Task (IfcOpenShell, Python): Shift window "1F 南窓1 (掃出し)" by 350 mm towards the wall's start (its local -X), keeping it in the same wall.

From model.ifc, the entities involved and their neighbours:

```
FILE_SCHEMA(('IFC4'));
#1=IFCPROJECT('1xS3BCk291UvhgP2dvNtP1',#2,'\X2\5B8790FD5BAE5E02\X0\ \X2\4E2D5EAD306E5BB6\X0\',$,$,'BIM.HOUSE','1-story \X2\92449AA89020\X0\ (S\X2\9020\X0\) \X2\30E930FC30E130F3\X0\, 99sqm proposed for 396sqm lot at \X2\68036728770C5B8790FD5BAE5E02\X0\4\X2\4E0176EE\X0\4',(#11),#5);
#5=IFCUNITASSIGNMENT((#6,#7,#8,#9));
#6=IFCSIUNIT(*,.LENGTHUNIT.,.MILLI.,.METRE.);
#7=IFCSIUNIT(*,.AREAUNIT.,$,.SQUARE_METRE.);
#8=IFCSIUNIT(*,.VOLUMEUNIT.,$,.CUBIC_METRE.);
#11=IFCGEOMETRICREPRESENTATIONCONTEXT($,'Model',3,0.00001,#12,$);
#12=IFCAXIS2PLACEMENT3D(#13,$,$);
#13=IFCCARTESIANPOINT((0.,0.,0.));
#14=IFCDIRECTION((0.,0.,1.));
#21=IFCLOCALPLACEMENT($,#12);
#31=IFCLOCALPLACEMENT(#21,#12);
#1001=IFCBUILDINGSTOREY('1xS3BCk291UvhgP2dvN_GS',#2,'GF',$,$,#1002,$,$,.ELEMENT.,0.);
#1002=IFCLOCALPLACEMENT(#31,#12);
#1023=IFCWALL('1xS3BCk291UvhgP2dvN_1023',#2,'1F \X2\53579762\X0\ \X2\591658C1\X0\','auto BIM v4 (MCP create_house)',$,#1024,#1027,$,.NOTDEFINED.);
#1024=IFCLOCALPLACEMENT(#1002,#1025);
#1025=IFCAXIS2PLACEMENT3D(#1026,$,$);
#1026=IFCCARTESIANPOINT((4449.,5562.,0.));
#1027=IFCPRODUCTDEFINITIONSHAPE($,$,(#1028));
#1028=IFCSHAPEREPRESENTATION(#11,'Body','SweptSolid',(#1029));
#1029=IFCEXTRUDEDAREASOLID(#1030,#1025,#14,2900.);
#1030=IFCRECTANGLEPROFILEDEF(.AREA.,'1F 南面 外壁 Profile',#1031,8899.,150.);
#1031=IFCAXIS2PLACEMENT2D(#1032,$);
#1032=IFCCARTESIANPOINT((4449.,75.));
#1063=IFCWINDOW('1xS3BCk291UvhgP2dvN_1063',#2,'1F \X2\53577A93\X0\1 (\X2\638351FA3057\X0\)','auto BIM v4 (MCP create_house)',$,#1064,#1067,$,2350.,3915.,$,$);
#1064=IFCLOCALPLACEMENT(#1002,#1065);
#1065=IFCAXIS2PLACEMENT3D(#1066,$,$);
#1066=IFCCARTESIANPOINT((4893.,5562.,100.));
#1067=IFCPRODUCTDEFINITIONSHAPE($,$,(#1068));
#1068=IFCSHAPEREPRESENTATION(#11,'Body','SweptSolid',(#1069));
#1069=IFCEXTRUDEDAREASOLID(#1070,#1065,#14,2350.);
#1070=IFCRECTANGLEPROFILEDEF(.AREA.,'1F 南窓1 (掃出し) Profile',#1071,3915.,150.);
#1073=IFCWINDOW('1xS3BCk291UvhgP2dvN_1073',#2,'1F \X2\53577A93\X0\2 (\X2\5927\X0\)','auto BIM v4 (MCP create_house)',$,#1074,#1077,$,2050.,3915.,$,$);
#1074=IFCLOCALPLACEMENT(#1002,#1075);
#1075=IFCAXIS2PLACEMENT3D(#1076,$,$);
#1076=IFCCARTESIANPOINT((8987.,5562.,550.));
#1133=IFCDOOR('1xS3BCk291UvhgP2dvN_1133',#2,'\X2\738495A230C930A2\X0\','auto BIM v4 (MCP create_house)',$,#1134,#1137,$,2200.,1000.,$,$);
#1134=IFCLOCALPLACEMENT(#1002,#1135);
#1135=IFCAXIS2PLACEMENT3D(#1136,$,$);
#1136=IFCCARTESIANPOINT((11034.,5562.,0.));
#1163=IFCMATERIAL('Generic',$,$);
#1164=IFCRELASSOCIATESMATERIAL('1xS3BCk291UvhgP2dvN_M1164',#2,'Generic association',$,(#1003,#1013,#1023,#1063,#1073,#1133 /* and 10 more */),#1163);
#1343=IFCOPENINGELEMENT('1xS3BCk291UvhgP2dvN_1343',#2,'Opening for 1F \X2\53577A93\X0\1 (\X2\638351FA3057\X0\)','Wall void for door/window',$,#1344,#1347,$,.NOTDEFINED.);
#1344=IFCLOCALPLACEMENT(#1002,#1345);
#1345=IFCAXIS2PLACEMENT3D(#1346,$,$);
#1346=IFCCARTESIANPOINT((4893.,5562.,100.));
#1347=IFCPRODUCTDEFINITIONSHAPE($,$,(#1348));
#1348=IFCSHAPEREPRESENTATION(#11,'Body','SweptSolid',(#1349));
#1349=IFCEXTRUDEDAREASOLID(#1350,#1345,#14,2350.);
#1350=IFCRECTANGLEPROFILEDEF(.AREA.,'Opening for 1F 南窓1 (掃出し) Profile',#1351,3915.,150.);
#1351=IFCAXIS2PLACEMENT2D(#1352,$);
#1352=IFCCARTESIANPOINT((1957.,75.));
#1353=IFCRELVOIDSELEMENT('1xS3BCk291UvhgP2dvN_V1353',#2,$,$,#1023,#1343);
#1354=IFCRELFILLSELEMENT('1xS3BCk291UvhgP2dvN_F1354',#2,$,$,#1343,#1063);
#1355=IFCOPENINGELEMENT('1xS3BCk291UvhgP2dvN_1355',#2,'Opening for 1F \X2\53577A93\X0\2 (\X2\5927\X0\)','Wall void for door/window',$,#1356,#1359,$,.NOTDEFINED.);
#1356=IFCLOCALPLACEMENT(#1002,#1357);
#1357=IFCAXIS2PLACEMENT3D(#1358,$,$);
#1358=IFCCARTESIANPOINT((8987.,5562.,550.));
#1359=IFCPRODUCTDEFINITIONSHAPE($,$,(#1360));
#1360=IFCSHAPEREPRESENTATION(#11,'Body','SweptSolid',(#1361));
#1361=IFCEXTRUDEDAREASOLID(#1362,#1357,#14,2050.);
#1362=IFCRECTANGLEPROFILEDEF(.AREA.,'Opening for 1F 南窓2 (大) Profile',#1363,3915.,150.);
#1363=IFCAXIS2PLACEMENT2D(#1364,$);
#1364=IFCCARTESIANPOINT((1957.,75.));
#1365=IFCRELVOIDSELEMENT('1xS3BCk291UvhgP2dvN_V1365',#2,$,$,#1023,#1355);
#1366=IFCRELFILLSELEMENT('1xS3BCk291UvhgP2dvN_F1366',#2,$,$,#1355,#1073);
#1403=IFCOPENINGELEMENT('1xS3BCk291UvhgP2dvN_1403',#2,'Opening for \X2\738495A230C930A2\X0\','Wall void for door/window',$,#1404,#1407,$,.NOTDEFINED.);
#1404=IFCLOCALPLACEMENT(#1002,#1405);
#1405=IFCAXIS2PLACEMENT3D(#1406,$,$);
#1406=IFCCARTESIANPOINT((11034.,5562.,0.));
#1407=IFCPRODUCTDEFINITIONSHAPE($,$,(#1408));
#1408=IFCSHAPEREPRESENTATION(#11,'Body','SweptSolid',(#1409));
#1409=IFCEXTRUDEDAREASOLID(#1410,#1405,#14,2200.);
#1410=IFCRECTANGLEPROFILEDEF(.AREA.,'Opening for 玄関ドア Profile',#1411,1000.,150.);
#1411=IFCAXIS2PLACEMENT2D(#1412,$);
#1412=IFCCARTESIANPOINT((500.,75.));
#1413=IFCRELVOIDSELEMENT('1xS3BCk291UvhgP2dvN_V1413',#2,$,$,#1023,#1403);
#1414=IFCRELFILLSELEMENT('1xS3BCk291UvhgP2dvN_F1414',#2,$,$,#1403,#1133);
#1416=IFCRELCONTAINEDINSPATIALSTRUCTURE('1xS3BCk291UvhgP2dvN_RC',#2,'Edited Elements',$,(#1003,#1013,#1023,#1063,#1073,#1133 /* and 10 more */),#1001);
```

```python
import ifcopenshell
import ifcopenshell.api.geometry
import ifcopenshell.util.placement
import ifcopenshell.util.unit

model = ifcopenshell.open("model.ifc")
unit_scale = ifcopenshell.util.unit.calculate_unit_scale(model)

window = model.by_guid("1xS3BCk291UvhgP2dvN_1063")
opening = window.FillsVoids[0].RelatingOpeningElement
wall = opening.VoidsElements[0].RelatingBuildingElement

wall_matrix = ifcopenshell.util.placement.get_local_placement(wall.ObjectPlacement)
shift = wall_matrix[:3, 0] * -0.35 / unit_scale
before = ifcopenshell.util.placement.get_local_placement(window.ObjectPlacement)[:3, 3].copy()

# The window is not placed relative to its opening, so move both.
for product in (opening, window):
    matrix = ifcopenshell.util.placement.get_local_placement(product.ObjectPlacement)
    matrix[:3, 3] += shift
    ifcopenshell.api.geometry.edit_object_placement(model, product=product, matrix=matrix, is_si=False)

after = ifcopenshell.util.placement.get_local_placement(window.ObjectPlacement)[:3, 3]
print("window moved by", (after - before).round(3) + 0.0)

model.write("model_rev.ifc")
```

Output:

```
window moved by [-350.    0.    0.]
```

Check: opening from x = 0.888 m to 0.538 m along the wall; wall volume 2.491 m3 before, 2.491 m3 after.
